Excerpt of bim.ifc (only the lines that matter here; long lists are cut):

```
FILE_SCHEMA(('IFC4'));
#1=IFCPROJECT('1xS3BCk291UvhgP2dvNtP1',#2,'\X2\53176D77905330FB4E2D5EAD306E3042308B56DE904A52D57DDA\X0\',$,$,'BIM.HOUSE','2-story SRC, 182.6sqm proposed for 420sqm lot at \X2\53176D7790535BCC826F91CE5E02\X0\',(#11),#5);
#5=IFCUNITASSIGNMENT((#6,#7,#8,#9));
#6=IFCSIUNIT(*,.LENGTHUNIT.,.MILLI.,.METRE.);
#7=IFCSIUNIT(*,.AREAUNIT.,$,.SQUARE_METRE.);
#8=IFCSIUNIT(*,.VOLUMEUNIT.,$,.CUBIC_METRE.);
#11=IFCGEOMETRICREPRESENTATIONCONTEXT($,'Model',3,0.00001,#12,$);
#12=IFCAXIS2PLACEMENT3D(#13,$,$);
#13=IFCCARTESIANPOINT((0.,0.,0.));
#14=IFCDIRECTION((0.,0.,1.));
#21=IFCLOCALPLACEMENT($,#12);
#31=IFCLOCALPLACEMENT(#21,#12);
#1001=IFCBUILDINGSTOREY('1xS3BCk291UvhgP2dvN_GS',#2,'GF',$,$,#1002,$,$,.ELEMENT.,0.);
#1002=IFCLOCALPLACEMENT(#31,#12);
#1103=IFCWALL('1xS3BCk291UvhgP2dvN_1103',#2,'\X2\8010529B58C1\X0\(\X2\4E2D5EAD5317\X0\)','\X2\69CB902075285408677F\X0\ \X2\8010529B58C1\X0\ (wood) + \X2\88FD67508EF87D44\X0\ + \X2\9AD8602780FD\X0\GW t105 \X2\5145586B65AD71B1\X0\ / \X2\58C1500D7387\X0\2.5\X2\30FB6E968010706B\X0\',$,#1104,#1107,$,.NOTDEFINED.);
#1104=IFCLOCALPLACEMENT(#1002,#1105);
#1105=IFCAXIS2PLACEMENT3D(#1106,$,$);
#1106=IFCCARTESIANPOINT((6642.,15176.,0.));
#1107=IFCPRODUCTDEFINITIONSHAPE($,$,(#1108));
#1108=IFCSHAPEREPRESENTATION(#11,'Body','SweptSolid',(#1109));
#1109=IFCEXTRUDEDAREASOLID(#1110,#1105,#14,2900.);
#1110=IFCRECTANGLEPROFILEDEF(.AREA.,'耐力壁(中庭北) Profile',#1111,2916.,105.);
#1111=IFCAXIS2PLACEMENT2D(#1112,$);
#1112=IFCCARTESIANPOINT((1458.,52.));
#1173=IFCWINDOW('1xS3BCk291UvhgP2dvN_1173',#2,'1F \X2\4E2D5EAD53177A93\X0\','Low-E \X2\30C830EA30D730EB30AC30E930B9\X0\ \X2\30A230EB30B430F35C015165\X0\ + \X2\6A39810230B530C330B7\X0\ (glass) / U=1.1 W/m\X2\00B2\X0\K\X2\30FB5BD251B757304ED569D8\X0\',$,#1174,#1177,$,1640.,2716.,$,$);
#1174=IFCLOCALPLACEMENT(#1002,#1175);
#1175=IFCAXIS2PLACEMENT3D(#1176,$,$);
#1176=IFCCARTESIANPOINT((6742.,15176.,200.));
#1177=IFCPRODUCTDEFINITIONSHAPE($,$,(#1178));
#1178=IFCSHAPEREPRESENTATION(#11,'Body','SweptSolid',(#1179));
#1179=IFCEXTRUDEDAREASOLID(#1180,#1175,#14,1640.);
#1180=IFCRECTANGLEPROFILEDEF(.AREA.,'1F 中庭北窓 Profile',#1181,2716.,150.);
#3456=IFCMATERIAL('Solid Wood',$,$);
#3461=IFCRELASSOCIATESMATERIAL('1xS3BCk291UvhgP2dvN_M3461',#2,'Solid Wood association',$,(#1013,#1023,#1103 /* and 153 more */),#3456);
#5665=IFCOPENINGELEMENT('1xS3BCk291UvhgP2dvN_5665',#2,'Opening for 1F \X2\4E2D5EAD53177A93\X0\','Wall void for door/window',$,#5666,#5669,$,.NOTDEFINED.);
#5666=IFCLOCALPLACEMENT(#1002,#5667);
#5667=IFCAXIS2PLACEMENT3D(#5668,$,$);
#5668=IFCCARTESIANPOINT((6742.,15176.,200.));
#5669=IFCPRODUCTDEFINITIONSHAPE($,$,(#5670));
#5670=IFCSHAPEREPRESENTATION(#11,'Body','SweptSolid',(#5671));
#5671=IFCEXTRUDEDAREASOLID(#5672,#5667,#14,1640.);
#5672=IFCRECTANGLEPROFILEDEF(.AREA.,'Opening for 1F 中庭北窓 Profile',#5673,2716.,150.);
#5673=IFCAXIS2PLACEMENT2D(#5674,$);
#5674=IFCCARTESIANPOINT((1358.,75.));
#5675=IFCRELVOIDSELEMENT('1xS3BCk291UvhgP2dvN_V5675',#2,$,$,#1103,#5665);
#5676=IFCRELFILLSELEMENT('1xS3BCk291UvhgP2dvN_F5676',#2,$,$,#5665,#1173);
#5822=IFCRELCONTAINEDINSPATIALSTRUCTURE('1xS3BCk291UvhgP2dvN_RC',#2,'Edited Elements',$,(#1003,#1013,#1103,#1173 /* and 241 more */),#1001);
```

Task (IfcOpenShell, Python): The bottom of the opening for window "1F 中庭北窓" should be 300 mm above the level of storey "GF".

```python
import numpy as np
import ifcopenshell
import ifcopenshell.api.geometry
import ifcopenshell.geom
import ifcopenshell.util.element
import ifcopenshell.util.placement
import ifcopenshell.util.shape
import ifcopenshell.util.unit

model = ifcopenshell.open("bim.ifc")
unit_scale = ifcopenshell.util.unit.calculate_unit_scale(model)

window = model.by_id(1173)
opening = window.FillsVoids[0].RelatingOpeningElement
storey = ifcopenshell.util.element.get_container(window, ifc_class="IfcBuildingStorey")
level = ifcopenshell.util.placement.get_local_placement(storey.ObjectPlacement)[2, 3]

# The opening's origin need not be at the sill, so measure its lowest point.
shape = ifcopenshell.geom.create_shape(ifcopenshell.geom.settings(), opening)
bottom = ifcopenshell.util.shape.get_shape_bottom_elevation(shape, shape.geometry) / unit_scale
dz = level + 0.3 / unit_scale - bottom

shift = np.array([0.0, 0.0, dz])
# The window is not placed relative to its opening, so move both.
for product in (opening, window):
    matrix = ifcopenshell.util.placement.get_local_placement(product.ObjectPlacement)
    matrix[:3, 3] += shift
    ifcopenshell.api.geometry.edit_object_placement(model, product=product, matrix=matrix, is_si=False)

print(f"moved by {dz * unit_scale:+.3f} m")

model.write("bim_rev.ifc")
```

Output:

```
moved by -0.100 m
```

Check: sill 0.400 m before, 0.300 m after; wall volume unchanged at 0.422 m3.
